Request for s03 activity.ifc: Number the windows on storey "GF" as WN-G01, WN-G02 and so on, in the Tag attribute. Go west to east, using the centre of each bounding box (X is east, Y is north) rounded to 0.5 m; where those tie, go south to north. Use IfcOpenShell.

First a look at what the model holds.

```python
import ifcopenshell
import ifcopenshell.util.element
import ifcopenshell.util.placement

model = ifcopenshell.open("s03 activity.ifc")
print(model.schema)
storey = next(s for s in model.by_type("IfcBuildingStorey") if s.Name == "GF")
windows = [e for e in ifcopenshell.util.element.get_decomposition(storey) if e.is_a("IfcWindow")]
for e in sorted(windows, key=lambda e: e.id()):
    origin = ifcopenshell.util.placement.get_local_placement(e.ObjectPlacement)[:3, 3]
    print(e.id(), e.Tag, e.Name, origin.round(2) + 0.0, sep=" | ")
```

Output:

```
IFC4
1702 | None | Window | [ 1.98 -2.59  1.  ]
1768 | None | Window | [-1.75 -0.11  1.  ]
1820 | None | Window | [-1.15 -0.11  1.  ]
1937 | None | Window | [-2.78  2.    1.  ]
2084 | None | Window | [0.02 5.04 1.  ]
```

```python
import ifcopenshell
import ifcopenshell.geom
import ifcopenshell.util.element
import ifcopenshell.util.shape

model = ifcopenshell.open("s03 activity.ifc")
settings = ifcopenshell.geom.settings()
settings.set("use-world-coords", True)


def centre(element):
    shape = ifcopenshell.geom.create_shape(settings, element)
    return ifcopenshell.util.shape.get_bbox_centroid(shape.geometry)


storey = next(s for s in model.by_type("IfcBuildingStorey") if s.Name == "GF")
windows = [e for e in ifcopenshell.util.element.get_decomposition(storey) if e.is_a("IfcWindow")]

# Insertion points can sit at a corner or the storey origin, so sort by the geometry (in metres).
centres = {e: centre(e) for e in windows}
windows.sort(key=lambda e: (round(centres[e][0] / 0.5), centres[e][1]))

for i, e in enumerate(windows, start=1):
    number = f"WN-G{i:02d}"
    e.Tag = number
    print(e.id(), number)

model.write("s03 activity_rev.ifc")
```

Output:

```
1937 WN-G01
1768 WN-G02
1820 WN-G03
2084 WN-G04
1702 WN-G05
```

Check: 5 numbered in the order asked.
